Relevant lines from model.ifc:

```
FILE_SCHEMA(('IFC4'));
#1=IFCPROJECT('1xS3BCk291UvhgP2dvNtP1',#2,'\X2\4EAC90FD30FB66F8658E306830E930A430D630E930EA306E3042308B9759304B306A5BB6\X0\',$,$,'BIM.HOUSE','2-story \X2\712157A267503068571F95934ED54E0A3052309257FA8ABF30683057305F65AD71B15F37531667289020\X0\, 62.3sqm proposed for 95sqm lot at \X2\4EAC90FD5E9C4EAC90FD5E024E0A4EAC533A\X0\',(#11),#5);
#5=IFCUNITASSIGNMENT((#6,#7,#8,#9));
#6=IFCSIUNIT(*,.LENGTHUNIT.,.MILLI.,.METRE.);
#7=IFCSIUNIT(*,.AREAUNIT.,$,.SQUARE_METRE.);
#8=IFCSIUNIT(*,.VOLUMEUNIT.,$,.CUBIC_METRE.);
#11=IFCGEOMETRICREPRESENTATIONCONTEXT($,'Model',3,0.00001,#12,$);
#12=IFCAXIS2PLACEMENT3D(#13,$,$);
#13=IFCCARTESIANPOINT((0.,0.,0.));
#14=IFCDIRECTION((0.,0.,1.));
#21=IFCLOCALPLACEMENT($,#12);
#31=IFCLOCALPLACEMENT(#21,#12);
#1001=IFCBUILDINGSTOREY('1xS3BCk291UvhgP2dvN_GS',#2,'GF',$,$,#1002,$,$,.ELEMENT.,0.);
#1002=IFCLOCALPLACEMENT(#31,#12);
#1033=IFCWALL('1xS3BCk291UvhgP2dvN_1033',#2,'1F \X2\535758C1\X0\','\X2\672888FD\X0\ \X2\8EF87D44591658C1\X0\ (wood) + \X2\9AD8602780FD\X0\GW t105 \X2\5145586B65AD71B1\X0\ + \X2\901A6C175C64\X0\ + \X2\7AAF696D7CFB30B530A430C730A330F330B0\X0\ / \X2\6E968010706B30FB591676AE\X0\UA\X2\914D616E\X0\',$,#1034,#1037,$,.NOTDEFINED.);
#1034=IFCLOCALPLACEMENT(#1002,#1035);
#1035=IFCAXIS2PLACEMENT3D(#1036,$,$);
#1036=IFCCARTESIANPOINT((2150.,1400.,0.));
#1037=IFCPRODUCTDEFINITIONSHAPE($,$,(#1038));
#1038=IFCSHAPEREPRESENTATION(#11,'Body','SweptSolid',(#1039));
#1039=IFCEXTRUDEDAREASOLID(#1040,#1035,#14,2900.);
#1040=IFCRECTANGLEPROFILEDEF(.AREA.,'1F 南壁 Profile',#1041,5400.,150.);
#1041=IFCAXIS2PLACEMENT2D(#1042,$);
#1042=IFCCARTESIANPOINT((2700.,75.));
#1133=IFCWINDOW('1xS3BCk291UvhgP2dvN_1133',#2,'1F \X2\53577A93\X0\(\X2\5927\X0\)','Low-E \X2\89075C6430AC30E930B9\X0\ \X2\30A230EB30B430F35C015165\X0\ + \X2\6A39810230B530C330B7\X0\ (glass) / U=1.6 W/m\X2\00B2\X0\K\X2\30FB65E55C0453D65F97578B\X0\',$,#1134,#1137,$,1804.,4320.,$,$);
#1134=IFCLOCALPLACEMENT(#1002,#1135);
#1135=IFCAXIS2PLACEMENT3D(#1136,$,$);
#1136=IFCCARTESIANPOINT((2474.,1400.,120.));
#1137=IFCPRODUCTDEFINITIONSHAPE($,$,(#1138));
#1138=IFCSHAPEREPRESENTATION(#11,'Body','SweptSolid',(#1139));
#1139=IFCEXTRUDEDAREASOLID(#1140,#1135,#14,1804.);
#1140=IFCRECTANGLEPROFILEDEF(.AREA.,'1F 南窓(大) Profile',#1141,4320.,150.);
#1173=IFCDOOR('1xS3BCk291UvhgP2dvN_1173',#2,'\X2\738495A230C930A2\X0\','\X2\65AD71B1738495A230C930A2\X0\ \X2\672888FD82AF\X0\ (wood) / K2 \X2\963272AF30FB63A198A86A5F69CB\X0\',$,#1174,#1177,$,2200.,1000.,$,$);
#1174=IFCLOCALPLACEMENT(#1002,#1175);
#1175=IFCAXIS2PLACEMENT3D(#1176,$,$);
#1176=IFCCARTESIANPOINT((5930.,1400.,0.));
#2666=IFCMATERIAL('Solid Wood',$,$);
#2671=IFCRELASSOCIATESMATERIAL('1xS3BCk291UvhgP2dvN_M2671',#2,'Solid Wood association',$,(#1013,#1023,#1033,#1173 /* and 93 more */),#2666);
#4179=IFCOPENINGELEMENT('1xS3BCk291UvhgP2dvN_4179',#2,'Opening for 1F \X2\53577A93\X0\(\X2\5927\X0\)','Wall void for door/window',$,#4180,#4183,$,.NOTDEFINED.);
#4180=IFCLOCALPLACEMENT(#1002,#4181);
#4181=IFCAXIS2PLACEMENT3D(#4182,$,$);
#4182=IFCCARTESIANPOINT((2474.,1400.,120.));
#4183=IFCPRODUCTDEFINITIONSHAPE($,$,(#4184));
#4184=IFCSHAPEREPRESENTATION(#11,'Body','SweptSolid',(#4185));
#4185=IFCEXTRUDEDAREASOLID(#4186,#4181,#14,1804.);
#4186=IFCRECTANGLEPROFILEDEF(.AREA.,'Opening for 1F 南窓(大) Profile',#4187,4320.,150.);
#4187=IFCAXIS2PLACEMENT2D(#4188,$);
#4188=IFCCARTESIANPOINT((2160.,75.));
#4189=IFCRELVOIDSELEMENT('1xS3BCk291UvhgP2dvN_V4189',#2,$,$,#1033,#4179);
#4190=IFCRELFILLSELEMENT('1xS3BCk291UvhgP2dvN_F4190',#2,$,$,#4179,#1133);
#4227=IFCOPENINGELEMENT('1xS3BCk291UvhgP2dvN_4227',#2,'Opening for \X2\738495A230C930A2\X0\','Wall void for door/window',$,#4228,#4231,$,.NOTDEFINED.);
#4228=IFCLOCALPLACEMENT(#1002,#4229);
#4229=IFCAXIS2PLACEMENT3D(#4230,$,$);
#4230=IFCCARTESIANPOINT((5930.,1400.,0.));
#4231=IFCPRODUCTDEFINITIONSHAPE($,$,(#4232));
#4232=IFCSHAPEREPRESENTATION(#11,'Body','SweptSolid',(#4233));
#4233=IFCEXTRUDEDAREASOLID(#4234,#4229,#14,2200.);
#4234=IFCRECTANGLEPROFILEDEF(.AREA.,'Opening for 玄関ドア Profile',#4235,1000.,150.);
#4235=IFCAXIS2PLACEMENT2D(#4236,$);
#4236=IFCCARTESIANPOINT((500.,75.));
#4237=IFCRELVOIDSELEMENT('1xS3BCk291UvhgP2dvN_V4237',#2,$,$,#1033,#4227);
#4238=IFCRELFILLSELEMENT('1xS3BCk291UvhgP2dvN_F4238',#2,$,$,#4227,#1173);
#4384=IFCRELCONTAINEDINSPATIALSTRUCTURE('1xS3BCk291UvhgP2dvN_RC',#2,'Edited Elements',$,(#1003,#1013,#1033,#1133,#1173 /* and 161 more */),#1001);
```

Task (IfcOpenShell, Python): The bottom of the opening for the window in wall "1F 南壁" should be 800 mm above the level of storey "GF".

```python
import numpy as np
import ifcopenshell
import ifcopenshell.api.geometry
import ifcopenshell.geom
import ifcopenshell.util.element
import ifcopenshell.util.placement
import ifcopenshell.util.shape
import ifcopenshell.util.unit

model = ifcopenshell.open("model.ifc")
unit_scale = ifcopenshell.util.unit.calculate_unit_scale(model)

window = model.by_guid("1xS3BCk291UvhgP2dvN_1133")
opening = window.FillsVoids[0].RelatingOpeningElement
storey = ifcopenshell.util.element.get_container(window, ifc_class="IfcBuildingStorey")
level = ifcopenshell.util.placement.get_local_placement(storey.ObjectPlacement)[2, 3]

# The opening's origin need not be at the sill, so measure its lowest point.
shape = ifcopenshell.geom.create_shape(ifcopenshell.geom.settings(), opening)
bottom = ifcopenshell.util.shape.get_shape_bottom_elevation(shape, shape.geometry) / unit_scale
dz = level + 0.8 / unit_scale - bottom

shift = np.array([0.0, 0.0, dz])
# The window is not placed relative to its opening, so move both.
for product in (opening, window):
    matrix = ifcopenshell.util.placement.get_local_placement(product.ObjectPlacement)
    matrix[:3, 3] += shift
    ifcopenshell.api.geometry.edit_object_placement(model, product=product, matrix=matrix, is_si=False)

print(f"moved by {dz * unit_scale:+.3f} m")

model.write("model_rev.ifc")
```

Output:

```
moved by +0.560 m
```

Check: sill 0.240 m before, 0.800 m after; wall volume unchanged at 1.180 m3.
